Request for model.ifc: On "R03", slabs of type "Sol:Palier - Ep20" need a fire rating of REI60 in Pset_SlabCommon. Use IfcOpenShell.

First a look at what the model holds.

```python
import ifcopenshell
import ifcopenshell.util.element

model = ifcopenshell.open("model.ifc")
print(model.schema)
storey = next(s for s in model.by_type("IfcBuildingStorey") if s.Name == "R03")
slabs = [e for e in ifcopenshell.util.element.get_decomposition(storey) if e.is_a("IfcSlab")]
seen = {}
for e in slabs:
    element_type = ifcopenshell.util.element.get_type(e)
    key = (element_type.Name if element_type != e and element_type else None, ifcopenshell.util.element.get_pset(e, "Pset_SlabCommon", "FireRating"))
    seen[key] = seen.get(key, 0) + 1
for (name, value), count in sorted(seen.items(), key=str):
    print(count, "x", name, "|", value)
```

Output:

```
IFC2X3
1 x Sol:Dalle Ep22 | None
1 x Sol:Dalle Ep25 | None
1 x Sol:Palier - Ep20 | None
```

```python
import ifcopenshell
import ifcopenshell.api.pset
import ifcopenshell.util.element

model = ifcopenshell.open("model.ifc")

storey = next(s for s in model.by_type("IfcBuildingStorey") if s.Name == "R03")
slabs = [e for e in ifcopenshell.util.element.get_decomposition(storey) if e.is_a("IfcSlab")]

count = 0
for e in slabs:
    element_type = ifcopenshell.util.element.get_type(e)
    if element_type in (None, e) or element_type.Name != "Sol:Palier - Ep20":
        continue
    # add_pset returns the element's existing set when there is one.
    pset = ifcopenshell.api.pset.add_pset(model, product=e, name="Pset_SlabCommon")
    ifcopenshell.api.pset.edit_pset(model, pset=pset, properties={"FireRating": "REI60"})
    count += 1

print(count, "slabs updated")

model.write("model_rev.ifc")
```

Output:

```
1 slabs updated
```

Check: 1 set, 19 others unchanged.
